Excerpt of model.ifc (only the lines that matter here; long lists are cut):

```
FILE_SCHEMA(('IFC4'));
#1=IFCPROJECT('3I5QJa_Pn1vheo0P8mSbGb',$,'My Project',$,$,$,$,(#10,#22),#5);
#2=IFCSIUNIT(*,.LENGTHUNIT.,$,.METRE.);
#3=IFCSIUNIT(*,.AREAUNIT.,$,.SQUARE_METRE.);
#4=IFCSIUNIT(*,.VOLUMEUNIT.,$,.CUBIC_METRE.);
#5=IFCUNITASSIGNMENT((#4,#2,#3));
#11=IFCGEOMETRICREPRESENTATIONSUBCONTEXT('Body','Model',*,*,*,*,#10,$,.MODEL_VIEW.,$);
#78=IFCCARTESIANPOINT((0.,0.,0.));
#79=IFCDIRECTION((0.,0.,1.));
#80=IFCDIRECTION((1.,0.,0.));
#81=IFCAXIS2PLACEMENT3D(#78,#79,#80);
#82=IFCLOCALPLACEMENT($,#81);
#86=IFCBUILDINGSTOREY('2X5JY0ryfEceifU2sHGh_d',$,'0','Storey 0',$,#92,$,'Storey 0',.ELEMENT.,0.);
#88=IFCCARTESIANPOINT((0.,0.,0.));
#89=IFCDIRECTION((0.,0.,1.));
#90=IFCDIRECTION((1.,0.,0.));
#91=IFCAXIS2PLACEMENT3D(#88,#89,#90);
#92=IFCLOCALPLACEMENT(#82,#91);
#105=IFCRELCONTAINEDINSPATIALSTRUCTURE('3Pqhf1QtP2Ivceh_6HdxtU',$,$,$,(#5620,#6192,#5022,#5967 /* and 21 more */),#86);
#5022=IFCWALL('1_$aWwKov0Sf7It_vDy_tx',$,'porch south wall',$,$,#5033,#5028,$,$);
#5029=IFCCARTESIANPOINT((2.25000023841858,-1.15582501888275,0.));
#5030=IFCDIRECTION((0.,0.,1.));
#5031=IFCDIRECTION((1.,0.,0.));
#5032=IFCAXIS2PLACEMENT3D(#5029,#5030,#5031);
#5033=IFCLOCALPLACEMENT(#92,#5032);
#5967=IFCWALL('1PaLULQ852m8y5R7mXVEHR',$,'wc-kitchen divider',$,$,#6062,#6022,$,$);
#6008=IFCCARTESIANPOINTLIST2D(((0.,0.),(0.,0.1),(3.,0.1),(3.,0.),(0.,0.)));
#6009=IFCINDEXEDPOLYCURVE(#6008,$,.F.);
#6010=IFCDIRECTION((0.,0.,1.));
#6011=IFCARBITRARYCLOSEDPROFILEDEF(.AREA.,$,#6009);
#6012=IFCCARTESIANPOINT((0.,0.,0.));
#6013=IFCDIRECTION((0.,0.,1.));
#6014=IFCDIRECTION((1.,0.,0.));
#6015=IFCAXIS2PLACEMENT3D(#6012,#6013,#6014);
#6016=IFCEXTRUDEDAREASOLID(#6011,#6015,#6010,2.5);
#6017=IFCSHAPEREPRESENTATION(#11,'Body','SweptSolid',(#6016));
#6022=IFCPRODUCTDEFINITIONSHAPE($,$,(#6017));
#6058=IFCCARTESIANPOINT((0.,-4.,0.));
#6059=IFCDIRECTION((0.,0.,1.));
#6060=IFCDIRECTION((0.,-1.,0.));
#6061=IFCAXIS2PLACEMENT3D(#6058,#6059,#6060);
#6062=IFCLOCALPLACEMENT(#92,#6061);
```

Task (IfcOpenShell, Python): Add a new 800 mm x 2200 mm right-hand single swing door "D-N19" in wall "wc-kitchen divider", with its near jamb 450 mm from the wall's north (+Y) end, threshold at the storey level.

```python
import numpy as np
import ifcopenshell
import ifcopenshell.api.feature
import ifcopenshell.api.geometry
import ifcopenshell.api.root
import ifcopenshell.api.spatial
import ifcopenshell.geom
import ifcopenshell.util.element
import ifcopenshell.util.placement
import ifcopenshell.util.representation
import ifcopenshell.util.shape
import ifcopenshell.util.unit

model = ifcopenshell.open("model.ifc")
unit_scale = ifcopenshell.util.unit.calculate_unit_scale(model)
settings = ifcopenshell.geom.settings()


def volume(element):
    """Net volume in cubic metres, openings subtracted."""
    shape = ifcopenshell.geom.create_shape(settings, element)
    return ifcopenshell.util.shape.get_volume(shape.geometry)


wall = model.by_guid("1PaLULQ852m8y5R7mXVEHR")
storey = ifcopenshell.util.element.get_container(wall, ifc_class="IfcBuildingStorey")
context = ifcopenshell.util.representation.get_context(model, "Model", "Body", "MODEL_VIEW")
before = volume(wall)

width, height, from_end, sill = 0.8, 2.2, 0.45, 0.0  # metres

# The wall runs along its own X axis, and the end named is its -X end.
wall_shape = ifcopenshell.geom.create_shape(settings, wall)
x, y, z = ifcopenshell.util.shape.get_vertices(wall_shape.geometry).T
start = x.min() + from_end
face, thickness = float(y.min()), float(y.max() - y.min())
wall_matrix = ifcopenshell.util.placement.get_local_placement(wall.ObjectPlacement)
level = ifcopenshell.util.placement.get_local_placement(storey.ObjectPlacement)[2, 3]


def in_wall(x, y):
    """Placement at x, y metres in the wall's axes, at sill height."""
    matrix = wall_matrix.copy()
    matrix[:, 3] = wall_matrix @ np.array([x / unit_scale, y / unit_scale, 0.0, 1.0])
    matrix[2, 3] = level + sill / unit_scale
    return matrix


# Opening: a box that overshoots both wall faces by 50 mm.
opening = ifcopenshell.api.root.create_entity(model, ifc_class="IfcOpeningElement", predefined_type="OPENING")
box = ifcopenshell.api.geometry.add_wall_representation(
    model, context=context, length=width, height=height, thickness=thickness + 0.1
)
ifcopenshell.api.geometry.assign_representation(model, product=opening, representation=box)
ifcopenshell.api.geometry.edit_object_placement(model, product=opening, matrix=in_wall(start, face - 0.05), is_si=False)
ifcopenshell.api.feature.add_feature(model, feature=opening, element=wall)

door = ifcopenshell.api.root.create_entity(model, ifc_class="IfcDoor", name="D-N19", predefined_type="DOOR")
door.OverallWidth, door.OverallHeight = width / unit_scale, height / unit_scale
door.OperationType = "SINGLE_SWING_RIGHT"
body = ifcopenshell.api.geometry.add_door_representation(
    model,
    context=context,
    overall_width=door.OverallWidth,
    overall_height=door.OverallHeight,
    operation_type="SINGLE_SWING_RIGHT",
    lining_properties={"LiningDepth": thickness / unit_scale, "ThresholdDepth": thickness / unit_scale},
)
ifcopenshell.api.geometry.assign_representation(model, product=door, representation=body)
ifcopenshell.api.spatial.assign_container(model, products=[door], relating_structure=storey)
ifcopenshell.api.feature.add_filling(model, opening=opening, element=door)

# The lining spans the wall, so the door starts at the wall face.
ifcopenshell.api.geometry.edit_object_placement(model, product=door, matrix=in_wall(start, face), is_si=False)

after = volume(wall)

print(f"wall volume {before:.3f} -> {after:.3f} m3")

model.write("model-out.ifc")
```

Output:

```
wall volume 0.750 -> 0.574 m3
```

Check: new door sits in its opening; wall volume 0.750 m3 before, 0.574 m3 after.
